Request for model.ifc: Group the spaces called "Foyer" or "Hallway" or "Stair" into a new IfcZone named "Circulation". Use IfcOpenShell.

First a look at what the model holds.

```python
import ifcopenshell

model = ifcopenshell.open("model.ifc")
print(model.schema)
seen = {}
for space in model.by_type("IfcSpace"):
    seen[space.LongName] = seen.get(space.LongName, 0) + 1
for name, count in sorted(seen.items(), key=str):
    print(count, "x", name)
print("zones:", [z.Name for z in model.by_type("IfcZone")][:20])
```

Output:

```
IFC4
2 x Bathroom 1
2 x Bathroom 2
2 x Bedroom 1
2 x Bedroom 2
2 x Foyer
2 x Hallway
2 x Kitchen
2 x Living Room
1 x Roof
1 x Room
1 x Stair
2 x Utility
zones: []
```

```python
import ifcopenshell
import ifcopenshell.api.group
import ifcopenshell.api.root

model = ifcopenshell.open("model.ifc")

names = {"Foyer", "Hallway", "Stair"}
spaces = [s for s in model.by_type("IfcSpace") if s.LongName in names]

zone = ifcopenshell.api.root.create_entity(model, ifc_class="IfcZone", name="Circulation")
ifcopenshell.api.group.assign_group(model, products=spaces, group=zone)
print(len(spaces), "spaces in", zone.Name)

model.write("model_updated.ifc")
```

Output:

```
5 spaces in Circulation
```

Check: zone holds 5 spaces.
